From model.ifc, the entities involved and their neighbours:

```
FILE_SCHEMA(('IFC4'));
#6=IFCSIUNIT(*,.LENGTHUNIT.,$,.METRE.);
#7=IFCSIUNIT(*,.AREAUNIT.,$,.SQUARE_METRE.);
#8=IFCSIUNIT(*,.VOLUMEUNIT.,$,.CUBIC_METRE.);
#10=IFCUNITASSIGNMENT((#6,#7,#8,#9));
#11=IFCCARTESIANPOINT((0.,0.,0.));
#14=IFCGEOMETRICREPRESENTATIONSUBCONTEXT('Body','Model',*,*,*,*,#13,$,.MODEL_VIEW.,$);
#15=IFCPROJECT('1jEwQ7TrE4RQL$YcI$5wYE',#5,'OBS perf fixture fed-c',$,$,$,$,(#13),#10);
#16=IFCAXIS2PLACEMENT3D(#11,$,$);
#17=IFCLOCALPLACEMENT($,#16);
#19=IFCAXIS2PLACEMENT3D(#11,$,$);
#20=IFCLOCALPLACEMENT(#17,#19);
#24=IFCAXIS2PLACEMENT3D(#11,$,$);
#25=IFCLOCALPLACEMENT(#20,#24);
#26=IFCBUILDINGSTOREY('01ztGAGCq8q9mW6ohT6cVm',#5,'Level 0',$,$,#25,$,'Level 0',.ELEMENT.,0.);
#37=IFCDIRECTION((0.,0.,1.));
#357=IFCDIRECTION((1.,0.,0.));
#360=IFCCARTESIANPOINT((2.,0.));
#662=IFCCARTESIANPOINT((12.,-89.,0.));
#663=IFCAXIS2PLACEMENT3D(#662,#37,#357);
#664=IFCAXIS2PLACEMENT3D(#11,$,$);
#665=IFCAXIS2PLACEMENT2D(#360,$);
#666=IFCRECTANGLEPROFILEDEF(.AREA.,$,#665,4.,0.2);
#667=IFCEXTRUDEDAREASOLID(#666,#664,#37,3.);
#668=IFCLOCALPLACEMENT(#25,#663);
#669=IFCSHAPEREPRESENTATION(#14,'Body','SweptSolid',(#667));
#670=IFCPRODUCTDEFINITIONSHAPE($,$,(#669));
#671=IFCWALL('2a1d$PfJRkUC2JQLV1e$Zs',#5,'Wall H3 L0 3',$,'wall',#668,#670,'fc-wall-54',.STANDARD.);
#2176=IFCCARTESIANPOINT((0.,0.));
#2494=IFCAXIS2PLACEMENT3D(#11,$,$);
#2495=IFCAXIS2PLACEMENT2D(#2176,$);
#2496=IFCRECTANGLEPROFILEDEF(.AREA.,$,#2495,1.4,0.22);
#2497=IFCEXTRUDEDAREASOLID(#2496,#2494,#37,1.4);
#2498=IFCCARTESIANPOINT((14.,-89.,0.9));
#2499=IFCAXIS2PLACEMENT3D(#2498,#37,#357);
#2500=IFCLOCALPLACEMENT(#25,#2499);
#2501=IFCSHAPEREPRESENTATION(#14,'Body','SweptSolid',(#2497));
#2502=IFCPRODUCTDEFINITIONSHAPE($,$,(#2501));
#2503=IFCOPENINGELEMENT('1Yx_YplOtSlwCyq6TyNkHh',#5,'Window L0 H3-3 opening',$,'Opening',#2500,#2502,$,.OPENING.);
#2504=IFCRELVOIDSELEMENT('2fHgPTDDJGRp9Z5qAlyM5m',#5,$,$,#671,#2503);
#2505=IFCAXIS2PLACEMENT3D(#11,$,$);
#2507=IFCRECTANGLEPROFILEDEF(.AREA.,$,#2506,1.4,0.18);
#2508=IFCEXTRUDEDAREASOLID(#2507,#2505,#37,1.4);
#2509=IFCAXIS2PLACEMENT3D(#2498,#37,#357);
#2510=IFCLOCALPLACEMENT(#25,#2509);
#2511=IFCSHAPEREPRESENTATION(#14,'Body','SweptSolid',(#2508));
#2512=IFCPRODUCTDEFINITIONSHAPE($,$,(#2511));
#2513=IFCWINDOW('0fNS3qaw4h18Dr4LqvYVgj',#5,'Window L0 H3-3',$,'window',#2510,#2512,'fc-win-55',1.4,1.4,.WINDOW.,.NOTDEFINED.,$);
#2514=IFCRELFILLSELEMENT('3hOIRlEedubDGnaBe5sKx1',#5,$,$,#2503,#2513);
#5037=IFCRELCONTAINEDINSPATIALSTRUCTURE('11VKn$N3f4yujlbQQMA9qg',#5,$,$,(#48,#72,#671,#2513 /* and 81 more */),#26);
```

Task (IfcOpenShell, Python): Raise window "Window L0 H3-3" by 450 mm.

```python
import numpy as np
import ifcopenshell
import ifcopenshell.api.geometry
import ifcopenshell.util.placement
import ifcopenshell.util.unit

model = ifcopenshell.open("model.ifc")
unit_scale = ifcopenshell.util.unit.calculate_unit_scale(model)

window = model.by_guid("0fNS3qaw4h18Dr4LqvYVgj")
opening = window.FillsVoids[0].RelatingOpeningElement
dz = 0.45

shift = np.array([0.0, 0.0, dz])
# The window is not placed relative to its opening, so move both.
for product in (opening, window):
    matrix = ifcopenshell.util.placement.get_local_placement(product.ObjectPlacement)
    matrix[:3, 3] += shift
    ifcopenshell.api.geometry.edit_object_placement(model, product=product, matrix=matrix, is_si=False)

print(f"moved by {dz * unit_scale:+.3f} m")

model.write("model_v2.ifc")
```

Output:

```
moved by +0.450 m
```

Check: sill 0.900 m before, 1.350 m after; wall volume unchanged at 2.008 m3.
